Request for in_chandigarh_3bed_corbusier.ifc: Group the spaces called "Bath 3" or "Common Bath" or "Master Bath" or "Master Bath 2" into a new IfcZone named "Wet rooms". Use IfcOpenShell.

First a look at what the model holds.

```python
import ifcopenshell

model = ifcopenshell.open("in_chandigarh_3bed_corbusier.ifc")
print(model.schema)
seen = {}
for space in model.by_type("IfcSpace"):
    seen[space.LongName] = seen.get(space.LongName, 0) + 1
for name, count in sorted(seen.items(), key=str):
    print(count, "x", name)
print("zones:", [z.Name for z in model.by_type("IfcZone")][:20])
```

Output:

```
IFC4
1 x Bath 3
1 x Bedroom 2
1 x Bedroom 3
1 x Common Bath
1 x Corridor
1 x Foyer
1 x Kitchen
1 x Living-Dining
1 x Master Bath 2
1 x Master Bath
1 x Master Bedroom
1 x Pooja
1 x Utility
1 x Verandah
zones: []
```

```python
import ifcopenshell
import ifcopenshell.api.group
import ifcopenshell.api.root

model = ifcopenshell.open("in_chandigarh_3bed_corbusier.ifc")

names = {"Bath 3", "Common Bath", "Master Bath", "Master Bath 2"}
spaces = [s for s in model.by_type("IfcSpace") if s.LongName in names]

zone = ifcopenshell.api.root.create_entity(model, ifc_class="IfcZone", name="Wet rooms")
ifcopenshell.api.group.assign_group(model, products=spaces, group=zone)
print(len(spaces), "spaces in", zone.Name)

model.write("in_chandigarh_3bed_corbusier_rev.ifc")
```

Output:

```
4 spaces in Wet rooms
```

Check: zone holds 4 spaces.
